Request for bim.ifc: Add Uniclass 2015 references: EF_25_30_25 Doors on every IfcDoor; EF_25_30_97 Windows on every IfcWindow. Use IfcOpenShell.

First a look at what the model holds.

```python
import ifcopenshell

model = ifcopenshell.open("bim.ifc")
print(model.schema)
print("classifications:", [c.Name for c in model.by_type("IfcClassification")])
for ifc_class in ("IfcDoor", "IfcRoof", "IfcStair", "IfcWall", "IfcWindow"):
    print(ifc_class, len(model.by_type(ifc_class)))
```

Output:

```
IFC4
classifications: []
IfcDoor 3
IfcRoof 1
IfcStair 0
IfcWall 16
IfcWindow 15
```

```python
import ifcopenshell
import ifcopenshell.api.classification

model = ifcopenshell.open("bim.ifc")

system = ifcopenshell.api.classification.add_classification(model, classification="Uniclass 2015")

codes = {
    "IfcDoor": ("EF_25_30_25", "Doors"),
    "IfcWindow": ("EF_25_30_97", "Windows"),
}
for ifc_class, (code, name) in codes.items():
    products = model.by_type(ifc_class)
    ifcopenshell.api.classification.add_reference(
        model, products=products, classification=system, identification=code, name=name
    )
    print(code, len(products))

model.write("bim_rev.ifc")
```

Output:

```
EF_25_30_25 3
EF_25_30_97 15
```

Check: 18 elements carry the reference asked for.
